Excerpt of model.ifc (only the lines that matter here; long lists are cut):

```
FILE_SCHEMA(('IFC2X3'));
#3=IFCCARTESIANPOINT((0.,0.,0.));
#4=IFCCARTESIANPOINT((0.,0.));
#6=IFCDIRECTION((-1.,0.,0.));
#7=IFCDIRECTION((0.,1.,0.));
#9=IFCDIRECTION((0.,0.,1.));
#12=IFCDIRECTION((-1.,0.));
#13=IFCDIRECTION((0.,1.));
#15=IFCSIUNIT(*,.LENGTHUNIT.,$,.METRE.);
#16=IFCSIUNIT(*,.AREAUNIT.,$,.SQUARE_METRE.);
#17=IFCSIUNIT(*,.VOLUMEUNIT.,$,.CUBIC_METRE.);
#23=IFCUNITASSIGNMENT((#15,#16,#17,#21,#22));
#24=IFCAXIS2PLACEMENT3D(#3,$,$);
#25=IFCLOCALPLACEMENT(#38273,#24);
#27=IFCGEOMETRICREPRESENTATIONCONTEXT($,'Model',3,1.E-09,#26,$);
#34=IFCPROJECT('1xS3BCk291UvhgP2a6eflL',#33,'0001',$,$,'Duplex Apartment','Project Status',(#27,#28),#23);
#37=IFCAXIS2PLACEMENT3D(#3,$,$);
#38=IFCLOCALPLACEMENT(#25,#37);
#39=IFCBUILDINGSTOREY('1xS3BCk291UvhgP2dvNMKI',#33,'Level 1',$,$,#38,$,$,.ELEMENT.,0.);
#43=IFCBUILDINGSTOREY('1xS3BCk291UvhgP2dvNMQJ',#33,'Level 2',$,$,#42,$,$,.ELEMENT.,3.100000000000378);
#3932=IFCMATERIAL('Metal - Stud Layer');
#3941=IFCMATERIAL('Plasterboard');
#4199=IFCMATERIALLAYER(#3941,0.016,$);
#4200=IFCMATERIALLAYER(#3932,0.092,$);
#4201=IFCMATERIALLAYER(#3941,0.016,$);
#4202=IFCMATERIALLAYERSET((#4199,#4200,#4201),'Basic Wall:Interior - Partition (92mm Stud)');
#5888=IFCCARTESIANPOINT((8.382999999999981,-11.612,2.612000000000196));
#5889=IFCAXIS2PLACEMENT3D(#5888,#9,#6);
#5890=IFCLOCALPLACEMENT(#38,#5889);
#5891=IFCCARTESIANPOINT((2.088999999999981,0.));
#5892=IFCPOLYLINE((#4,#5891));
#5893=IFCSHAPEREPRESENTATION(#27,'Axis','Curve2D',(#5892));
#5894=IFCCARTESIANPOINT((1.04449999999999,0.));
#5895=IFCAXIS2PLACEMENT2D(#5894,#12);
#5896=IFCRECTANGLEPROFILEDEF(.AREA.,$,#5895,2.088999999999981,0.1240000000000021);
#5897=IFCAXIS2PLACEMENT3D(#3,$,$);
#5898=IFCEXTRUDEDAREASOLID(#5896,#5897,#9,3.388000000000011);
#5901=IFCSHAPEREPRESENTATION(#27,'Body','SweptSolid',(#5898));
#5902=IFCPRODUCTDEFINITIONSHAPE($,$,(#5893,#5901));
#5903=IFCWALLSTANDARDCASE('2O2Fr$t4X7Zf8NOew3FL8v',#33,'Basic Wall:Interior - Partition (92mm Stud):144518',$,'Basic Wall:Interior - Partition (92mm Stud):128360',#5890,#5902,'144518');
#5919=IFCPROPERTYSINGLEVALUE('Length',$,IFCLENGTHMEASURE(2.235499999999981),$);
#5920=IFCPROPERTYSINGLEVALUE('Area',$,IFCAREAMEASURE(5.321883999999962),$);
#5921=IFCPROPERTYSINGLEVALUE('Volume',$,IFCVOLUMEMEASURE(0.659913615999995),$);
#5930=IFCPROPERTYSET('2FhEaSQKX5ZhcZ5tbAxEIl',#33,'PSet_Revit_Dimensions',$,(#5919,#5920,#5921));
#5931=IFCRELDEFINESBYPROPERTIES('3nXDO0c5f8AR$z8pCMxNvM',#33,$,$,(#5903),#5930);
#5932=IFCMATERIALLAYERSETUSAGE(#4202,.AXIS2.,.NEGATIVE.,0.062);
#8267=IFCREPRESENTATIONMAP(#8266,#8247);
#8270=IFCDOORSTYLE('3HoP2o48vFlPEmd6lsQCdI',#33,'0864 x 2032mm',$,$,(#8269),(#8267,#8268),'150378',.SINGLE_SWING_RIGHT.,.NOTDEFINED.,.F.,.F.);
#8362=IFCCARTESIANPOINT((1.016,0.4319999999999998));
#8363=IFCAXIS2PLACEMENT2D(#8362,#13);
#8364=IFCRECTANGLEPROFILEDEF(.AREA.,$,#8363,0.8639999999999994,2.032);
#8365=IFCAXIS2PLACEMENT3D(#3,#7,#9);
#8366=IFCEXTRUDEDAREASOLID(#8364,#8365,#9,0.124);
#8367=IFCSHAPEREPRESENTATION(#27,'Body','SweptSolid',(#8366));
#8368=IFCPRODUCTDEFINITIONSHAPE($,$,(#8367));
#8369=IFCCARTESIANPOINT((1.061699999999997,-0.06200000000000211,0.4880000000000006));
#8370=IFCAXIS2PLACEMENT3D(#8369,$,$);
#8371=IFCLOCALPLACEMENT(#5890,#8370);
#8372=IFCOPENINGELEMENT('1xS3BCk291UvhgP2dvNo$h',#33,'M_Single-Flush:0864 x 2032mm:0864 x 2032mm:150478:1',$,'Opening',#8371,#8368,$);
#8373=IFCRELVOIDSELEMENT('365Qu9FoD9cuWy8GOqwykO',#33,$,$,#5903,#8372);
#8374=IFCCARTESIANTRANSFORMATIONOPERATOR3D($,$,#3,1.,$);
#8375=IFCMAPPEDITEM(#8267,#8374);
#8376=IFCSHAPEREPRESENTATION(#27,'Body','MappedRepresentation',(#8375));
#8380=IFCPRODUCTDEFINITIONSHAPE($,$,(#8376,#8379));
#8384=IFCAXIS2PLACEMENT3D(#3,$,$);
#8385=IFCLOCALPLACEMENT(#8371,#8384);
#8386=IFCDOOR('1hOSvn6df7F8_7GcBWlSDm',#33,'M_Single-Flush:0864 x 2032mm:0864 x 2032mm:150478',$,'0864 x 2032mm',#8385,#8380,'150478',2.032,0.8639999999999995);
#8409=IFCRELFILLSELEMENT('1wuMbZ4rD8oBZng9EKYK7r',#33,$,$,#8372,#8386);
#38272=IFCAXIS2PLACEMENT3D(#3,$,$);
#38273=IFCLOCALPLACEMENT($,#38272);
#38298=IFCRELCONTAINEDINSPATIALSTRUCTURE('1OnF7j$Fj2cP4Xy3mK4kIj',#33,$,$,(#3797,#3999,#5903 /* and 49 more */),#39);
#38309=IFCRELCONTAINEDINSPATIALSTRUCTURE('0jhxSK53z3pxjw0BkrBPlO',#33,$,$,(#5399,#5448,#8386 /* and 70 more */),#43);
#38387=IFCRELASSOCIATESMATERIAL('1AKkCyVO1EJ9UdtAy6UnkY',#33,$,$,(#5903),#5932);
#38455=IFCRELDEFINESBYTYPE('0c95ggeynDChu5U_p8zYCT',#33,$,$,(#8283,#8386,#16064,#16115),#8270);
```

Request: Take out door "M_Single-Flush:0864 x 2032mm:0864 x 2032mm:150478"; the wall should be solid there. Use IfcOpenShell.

```python
import ifcopenshell
import ifcopenshell.api.feature
import ifcopenshell.api.pset
import ifcopenshell.api.root
import ifcopenshell.geom
import ifcopenshell.util.element
import ifcopenshell.util.shape
import ifcopenshell.util.unit

model = ifcopenshell.open("model.ifc")
area_scale = ifcopenshell.util.unit.calculate_unit_scale(model, "AREAUNIT")
volume_scale = ifcopenshell.util.unit.calculate_unit_scale(model, "VOLUMEUNIT")
settings = ifcopenshell.geom.settings()


def volume(element):
    """Net volume in cubic metres, openings subtracted."""
    shape = ifcopenshell.geom.create_shape(settings, element)
    return ifcopenshell.util.shape.get_volume(shape.geometry)


door = model.by_guid("1hOSvn6df7F8_7GcBWlSDm")
opening = door.FillsVoids[0].RelatingOpeningElement
wall = opening.VoidsElements[0].RelatingBuildingElement
before = volume(wall)

ifcopenshell.api.root.remove_product(model, product=door)
ifcopenshell.api.feature.remove_feature(model, feature=opening)

after = volume(wall)
thickness = 0.124  # wall thickness in metres

# Update the wall's stored quantities.
pset = model.by_id(ifcopenshell.util.element.get_pset(wall, "PSet_Revit_Dimensions", should_inherit=False)["id"])
ifcopenshell.api.pset.edit_pset(model, pset=pset, properties={
    "Area": model.create_entity("IfcAreaMeasure", after / thickness / area_scale),
    "Volume": model.create_entity("IfcVolumeMeasure", after / volume_scale),
})

print(f"wall volume {before:.3f} -> {after:.3f} m3")

model.write("model_rev.ifc")
```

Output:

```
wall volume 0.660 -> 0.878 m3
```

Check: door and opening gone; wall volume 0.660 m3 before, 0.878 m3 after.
